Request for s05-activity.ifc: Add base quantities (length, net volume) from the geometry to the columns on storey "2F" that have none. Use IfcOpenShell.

First a look at what the model holds.

```python
import ifcopenshell
import ifcopenshell.util.element
import ifcopenshell.util.unit

model = ifcopenshell.open("s05-activity.ifc")
print(model.schema)
for unit_type in ("LENGTHUNIT", "AREAUNIT", "VOLUMEUNIT"):
    print(unit_type, ifcopenshell.util.unit.calculate_unit_scale(model, unit_type))
storey = next(s for s in model.by_type("IfcBuildingStorey") if s.Name == "2F")
columns = [e for e in ifcopenshell.util.element.get_decomposition(storey) if e.is_a("IfcColumn")]
for e in sorted(columns, key=lambda e: e.id()):
    print(e.id(), e.is_a(), e.Name, list(ifcopenshell.util.element.get_psets(e, qtos_only=True)), sep=" | ")
```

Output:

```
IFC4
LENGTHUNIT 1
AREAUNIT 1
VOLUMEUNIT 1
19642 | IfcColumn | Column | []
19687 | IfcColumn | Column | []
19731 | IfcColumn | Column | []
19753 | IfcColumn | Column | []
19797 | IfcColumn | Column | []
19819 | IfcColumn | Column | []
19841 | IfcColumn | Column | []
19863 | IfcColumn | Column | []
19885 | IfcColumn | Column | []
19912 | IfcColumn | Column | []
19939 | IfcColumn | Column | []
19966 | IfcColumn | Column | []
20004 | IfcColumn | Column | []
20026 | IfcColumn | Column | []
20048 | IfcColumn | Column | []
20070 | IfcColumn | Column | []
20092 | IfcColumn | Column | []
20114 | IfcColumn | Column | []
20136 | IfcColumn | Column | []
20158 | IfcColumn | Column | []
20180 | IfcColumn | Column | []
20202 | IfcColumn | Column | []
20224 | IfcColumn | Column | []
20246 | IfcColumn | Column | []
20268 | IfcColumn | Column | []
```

```python
import ifcopenshell
import ifcopenshell.api.pset
import ifcopenshell.geom
import ifcopenshell.util.element
import ifcopenshell.util.shape
import ifcopenshell.util.unit

model = ifcopenshell.open("s05-activity.ifc")
unit_scale = ifcopenshell.util.unit.calculate_unit_scale(model)
volume_scale = ifcopenshell.util.unit.calculate_unit_scale(model, "VOLUMEUNIT")
settings = ifcopenshell.geom.settings()

storey = next(s for s in model.by_type("IfcBuildingStorey") if s.Name == "2F")
columns = [e for e in ifcopenshell.util.element.get_decomposition(storey) if e.is_a("IfcColumn")]

for e in sorted(columns, key=lambda e: e.id()):
    if ifcopenshell.util.element.get_psets(e, qtos_only=True, should_inherit=False):
        continue
    # Geometry comes back in metres, in the element's own axes.
    shape = ifcopenshell.geom.create_shape(settings, e)
    values = {
        "Length": ifcopenshell.util.shape.get_z(shape.geometry) / unit_scale,
        "NetVolume": ifcopenshell.util.shape.get_volume(shape.geometry) / volume_scale,
    }
    qto = ifcopenshell.api.pset.add_qto(model, product=e, name="Qto_ColumnBaseQuantities")
    ifcopenshell.api.pset.edit_qto(model, qto=qto, properties=values)
    print(e.id(), {k: round(v, 3) for k, v in values.items()})

model.write("s05-activity_rev.ifc")
```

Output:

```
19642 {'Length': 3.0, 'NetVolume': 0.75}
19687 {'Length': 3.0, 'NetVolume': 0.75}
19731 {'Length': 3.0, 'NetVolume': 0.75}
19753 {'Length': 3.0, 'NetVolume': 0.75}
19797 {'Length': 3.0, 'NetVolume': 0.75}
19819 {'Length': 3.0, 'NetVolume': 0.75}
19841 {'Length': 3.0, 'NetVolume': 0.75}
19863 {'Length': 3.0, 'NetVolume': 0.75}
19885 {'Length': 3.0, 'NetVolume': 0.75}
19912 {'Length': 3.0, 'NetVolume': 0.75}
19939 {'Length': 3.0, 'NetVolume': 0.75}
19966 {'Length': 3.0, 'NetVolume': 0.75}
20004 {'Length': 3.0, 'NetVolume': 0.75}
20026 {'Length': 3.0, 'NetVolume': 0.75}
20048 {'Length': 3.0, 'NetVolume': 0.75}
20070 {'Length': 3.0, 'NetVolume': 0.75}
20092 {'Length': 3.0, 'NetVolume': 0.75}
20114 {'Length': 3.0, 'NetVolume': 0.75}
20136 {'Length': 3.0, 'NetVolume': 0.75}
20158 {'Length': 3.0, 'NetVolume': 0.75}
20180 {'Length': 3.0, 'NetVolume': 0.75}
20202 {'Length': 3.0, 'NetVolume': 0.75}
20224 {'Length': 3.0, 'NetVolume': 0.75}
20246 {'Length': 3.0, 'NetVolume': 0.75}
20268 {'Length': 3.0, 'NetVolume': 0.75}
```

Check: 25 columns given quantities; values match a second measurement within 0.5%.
